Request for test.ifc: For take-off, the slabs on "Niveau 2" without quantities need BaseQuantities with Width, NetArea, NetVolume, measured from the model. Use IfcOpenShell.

First a look at what the model holds.

```python
import ifcopenshell
import ifcopenshell.util.element
import ifcopenshell.util.unit

model = ifcopenshell.open("test.ifc")
print(model.schema)
for unit_type in ("LENGTHUNIT", "AREAUNIT", "VOLUMEUNIT"):
    print(unit_type, ifcopenshell.util.unit.calculate_unit_scale(model, unit_type))
storey = next(s for s in model.by_type("IfcBuildingStorey") if s.Name == "Niveau 2")
slabs = [e for e in ifcopenshell.util.element.get_decomposition(storey) if e.is_a("IfcSlab")]
for e in sorted(slabs, key=lambda e: e.id()):
    print(e.id(), e.is_a(), e.Name, list(ifcopenshell.util.element.get_psets(e, qtos_only=True)), sep=" | ")
```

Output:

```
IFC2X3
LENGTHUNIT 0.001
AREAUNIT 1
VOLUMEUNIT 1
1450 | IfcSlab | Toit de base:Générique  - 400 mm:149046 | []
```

```python
import ifcopenshell
import ifcopenshell.api.pset
import ifcopenshell.geom
import ifcopenshell.util.element
import ifcopenshell.util.shape
import ifcopenshell.util.unit

model = ifcopenshell.open("test.ifc")
unit_scale = ifcopenshell.util.unit.calculate_unit_scale(model)
area_scale = ifcopenshell.util.unit.calculate_unit_scale(model, "AREAUNIT")
volume_scale = ifcopenshell.util.unit.calculate_unit_scale(model, "VOLUMEUNIT")
settings = ifcopenshell.geom.settings()

storey = next(s for s in model.by_type("IfcBuildingStorey") if s.Name == "Niveau 2")
slabs = [e for e in ifcopenshell.util.element.get_decomposition(storey) if e.is_a("IfcSlab")]

for e in sorted(slabs, key=lambda e: e.id()):
    if ifcopenshell.util.element.get_psets(e, qtos_only=True, should_inherit=False):
        continue
    # Geometry comes back in metres, in the element's own axes.
    shape = ifcopenshell.geom.create_shape(settings, e)
    values = {
        "Width": ifcopenshell.util.shape.get_z(shape.geometry) / unit_scale,
        "NetArea": ifcopenshell.util.shape.get_footprint_area(shape.geometry) / area_scale,
        "NetVolume": ifcopenshell.util.shape.get_volume(shape.geometry) / volume_scale,
    }
    qto = ifcopenshell.api.pset.add_qto(model, product=e, name="BaseQuantities")
    ifcopenshell.api.pset.edit_qto(model, qto=qto, properties=values)
    print(e.id(), {k: round(v, 3) for k, v in values.items()})

model.write("test_edited.ifc")
```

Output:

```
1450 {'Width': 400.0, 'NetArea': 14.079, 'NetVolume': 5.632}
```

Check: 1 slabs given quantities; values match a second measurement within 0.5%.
